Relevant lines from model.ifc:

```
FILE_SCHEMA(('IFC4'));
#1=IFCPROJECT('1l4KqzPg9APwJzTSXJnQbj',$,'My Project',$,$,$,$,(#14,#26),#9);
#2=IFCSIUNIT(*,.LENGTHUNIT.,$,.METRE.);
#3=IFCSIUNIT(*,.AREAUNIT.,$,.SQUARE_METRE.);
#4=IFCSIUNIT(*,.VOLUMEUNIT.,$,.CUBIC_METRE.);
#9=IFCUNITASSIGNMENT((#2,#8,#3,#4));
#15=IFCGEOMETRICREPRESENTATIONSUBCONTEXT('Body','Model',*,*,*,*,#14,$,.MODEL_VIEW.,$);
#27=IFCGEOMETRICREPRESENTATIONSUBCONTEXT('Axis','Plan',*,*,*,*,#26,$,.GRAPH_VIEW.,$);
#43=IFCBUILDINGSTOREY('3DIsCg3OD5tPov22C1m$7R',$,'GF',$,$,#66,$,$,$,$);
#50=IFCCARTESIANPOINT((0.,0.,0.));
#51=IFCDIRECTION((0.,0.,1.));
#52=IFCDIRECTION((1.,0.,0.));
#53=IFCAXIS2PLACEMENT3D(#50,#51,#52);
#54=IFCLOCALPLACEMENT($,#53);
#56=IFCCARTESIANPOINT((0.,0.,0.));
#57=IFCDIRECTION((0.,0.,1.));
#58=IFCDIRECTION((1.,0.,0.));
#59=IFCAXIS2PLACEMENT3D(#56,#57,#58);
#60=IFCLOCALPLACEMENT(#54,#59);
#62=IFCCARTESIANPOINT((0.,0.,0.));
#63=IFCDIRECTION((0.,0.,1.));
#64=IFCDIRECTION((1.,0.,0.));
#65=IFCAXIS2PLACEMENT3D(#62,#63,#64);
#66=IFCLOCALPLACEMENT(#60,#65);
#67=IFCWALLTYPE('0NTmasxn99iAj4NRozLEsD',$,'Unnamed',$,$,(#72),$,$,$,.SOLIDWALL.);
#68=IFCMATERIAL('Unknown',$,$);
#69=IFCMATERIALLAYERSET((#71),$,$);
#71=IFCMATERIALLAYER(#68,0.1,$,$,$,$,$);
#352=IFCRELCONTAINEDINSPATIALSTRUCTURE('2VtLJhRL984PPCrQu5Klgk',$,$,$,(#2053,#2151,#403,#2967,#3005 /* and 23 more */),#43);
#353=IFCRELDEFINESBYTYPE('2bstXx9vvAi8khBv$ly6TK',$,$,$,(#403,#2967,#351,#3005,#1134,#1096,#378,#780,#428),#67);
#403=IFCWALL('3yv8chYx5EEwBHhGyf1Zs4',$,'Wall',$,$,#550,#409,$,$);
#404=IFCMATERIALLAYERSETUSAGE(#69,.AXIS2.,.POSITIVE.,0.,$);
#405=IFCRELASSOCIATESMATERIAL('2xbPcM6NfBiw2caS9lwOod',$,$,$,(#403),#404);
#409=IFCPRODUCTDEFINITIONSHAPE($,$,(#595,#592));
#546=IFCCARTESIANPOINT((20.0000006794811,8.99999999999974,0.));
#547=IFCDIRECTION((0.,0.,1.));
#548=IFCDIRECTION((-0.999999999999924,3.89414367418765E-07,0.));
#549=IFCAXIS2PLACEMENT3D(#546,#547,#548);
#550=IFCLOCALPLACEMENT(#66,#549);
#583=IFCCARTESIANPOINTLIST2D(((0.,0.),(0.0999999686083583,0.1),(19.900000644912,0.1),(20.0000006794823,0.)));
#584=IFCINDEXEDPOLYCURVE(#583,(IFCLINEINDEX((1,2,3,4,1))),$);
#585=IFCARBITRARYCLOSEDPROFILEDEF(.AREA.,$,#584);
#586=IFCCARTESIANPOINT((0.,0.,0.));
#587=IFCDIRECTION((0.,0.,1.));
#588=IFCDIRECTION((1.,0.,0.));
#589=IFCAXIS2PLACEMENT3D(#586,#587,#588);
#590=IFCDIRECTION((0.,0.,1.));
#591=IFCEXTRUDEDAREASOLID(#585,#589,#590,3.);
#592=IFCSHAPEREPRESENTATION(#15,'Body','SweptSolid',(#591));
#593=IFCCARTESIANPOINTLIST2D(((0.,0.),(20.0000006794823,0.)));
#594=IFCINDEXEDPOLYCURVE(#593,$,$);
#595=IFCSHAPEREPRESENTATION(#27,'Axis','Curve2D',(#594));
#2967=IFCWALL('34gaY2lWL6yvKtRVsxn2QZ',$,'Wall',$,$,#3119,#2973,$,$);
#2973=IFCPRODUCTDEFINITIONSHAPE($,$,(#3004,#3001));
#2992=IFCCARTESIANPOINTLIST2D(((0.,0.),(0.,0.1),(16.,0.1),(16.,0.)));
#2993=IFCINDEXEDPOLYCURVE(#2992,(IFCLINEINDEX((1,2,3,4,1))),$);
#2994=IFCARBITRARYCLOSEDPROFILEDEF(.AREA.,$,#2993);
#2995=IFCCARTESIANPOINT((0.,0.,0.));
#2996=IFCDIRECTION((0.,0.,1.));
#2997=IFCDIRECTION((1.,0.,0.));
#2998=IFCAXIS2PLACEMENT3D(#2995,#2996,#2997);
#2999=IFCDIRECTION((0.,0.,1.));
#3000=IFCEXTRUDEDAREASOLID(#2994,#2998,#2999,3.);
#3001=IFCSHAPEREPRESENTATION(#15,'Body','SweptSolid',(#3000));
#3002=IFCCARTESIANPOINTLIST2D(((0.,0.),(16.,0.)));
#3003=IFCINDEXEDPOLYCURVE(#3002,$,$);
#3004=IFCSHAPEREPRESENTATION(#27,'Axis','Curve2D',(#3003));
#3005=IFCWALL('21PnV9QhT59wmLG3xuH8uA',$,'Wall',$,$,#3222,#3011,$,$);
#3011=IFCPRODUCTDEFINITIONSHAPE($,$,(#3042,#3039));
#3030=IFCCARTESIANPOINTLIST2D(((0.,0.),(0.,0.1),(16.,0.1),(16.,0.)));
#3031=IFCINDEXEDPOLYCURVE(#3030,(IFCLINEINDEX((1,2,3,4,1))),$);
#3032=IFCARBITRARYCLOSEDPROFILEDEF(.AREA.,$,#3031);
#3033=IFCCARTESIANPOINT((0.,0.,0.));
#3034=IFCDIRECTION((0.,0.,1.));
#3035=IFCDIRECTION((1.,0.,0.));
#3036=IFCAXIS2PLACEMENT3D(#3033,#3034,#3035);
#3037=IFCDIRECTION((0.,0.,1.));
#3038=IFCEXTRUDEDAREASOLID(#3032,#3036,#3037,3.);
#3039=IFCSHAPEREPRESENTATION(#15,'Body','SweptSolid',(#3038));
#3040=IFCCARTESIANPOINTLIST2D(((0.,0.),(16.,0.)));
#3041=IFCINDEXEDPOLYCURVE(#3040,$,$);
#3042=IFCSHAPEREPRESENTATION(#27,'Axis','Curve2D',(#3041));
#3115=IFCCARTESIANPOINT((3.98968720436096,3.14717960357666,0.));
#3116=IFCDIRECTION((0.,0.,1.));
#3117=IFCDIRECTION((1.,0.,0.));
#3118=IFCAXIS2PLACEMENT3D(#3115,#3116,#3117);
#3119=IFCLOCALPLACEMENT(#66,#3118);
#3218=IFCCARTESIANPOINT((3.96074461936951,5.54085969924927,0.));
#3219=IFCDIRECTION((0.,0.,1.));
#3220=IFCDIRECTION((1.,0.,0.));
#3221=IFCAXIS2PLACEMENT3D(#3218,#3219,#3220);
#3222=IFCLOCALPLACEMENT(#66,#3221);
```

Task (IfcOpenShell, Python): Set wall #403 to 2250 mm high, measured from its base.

```python
import ifcopenshell
import ifcopenshell.geom
import ifcopenshell.util.representation
import ifcopenshell.util.shape
import ifcopenshell.util.unit

model = ifcopenshell.open("model.ifc")
unit_scale = ifcopenshell.util.unit.calculate_unit_scale(model)
settings = ifcopenshell.geom.settings()


def volume(element):
    """Net volume in cubic metres, openings subtracted."""
    shape = ifcopenshell.geom.create_shape(settings, element)
    return ifcopenshell.util.shape.get_volume(shape.geometry)


wall = model.by_guid("3yv8chYx5EEwBHhGyf1Zs4")
before = volume(wall)

body = ifcopenshell.util.representation.get_representation(wall, "Model", "Body")
solid = body.Items[0]
old_height = solid.Depth
solid.Depth = 2.25 / unit_scale
after = volume(wall)

print(f"height {old_height:g} -> {solid.Depth:g}, volume {before:.3f} -> {after:.3f} m3")

model.write("model-out.ifc")
```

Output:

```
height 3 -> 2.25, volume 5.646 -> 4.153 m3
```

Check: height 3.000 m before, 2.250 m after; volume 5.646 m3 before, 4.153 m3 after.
